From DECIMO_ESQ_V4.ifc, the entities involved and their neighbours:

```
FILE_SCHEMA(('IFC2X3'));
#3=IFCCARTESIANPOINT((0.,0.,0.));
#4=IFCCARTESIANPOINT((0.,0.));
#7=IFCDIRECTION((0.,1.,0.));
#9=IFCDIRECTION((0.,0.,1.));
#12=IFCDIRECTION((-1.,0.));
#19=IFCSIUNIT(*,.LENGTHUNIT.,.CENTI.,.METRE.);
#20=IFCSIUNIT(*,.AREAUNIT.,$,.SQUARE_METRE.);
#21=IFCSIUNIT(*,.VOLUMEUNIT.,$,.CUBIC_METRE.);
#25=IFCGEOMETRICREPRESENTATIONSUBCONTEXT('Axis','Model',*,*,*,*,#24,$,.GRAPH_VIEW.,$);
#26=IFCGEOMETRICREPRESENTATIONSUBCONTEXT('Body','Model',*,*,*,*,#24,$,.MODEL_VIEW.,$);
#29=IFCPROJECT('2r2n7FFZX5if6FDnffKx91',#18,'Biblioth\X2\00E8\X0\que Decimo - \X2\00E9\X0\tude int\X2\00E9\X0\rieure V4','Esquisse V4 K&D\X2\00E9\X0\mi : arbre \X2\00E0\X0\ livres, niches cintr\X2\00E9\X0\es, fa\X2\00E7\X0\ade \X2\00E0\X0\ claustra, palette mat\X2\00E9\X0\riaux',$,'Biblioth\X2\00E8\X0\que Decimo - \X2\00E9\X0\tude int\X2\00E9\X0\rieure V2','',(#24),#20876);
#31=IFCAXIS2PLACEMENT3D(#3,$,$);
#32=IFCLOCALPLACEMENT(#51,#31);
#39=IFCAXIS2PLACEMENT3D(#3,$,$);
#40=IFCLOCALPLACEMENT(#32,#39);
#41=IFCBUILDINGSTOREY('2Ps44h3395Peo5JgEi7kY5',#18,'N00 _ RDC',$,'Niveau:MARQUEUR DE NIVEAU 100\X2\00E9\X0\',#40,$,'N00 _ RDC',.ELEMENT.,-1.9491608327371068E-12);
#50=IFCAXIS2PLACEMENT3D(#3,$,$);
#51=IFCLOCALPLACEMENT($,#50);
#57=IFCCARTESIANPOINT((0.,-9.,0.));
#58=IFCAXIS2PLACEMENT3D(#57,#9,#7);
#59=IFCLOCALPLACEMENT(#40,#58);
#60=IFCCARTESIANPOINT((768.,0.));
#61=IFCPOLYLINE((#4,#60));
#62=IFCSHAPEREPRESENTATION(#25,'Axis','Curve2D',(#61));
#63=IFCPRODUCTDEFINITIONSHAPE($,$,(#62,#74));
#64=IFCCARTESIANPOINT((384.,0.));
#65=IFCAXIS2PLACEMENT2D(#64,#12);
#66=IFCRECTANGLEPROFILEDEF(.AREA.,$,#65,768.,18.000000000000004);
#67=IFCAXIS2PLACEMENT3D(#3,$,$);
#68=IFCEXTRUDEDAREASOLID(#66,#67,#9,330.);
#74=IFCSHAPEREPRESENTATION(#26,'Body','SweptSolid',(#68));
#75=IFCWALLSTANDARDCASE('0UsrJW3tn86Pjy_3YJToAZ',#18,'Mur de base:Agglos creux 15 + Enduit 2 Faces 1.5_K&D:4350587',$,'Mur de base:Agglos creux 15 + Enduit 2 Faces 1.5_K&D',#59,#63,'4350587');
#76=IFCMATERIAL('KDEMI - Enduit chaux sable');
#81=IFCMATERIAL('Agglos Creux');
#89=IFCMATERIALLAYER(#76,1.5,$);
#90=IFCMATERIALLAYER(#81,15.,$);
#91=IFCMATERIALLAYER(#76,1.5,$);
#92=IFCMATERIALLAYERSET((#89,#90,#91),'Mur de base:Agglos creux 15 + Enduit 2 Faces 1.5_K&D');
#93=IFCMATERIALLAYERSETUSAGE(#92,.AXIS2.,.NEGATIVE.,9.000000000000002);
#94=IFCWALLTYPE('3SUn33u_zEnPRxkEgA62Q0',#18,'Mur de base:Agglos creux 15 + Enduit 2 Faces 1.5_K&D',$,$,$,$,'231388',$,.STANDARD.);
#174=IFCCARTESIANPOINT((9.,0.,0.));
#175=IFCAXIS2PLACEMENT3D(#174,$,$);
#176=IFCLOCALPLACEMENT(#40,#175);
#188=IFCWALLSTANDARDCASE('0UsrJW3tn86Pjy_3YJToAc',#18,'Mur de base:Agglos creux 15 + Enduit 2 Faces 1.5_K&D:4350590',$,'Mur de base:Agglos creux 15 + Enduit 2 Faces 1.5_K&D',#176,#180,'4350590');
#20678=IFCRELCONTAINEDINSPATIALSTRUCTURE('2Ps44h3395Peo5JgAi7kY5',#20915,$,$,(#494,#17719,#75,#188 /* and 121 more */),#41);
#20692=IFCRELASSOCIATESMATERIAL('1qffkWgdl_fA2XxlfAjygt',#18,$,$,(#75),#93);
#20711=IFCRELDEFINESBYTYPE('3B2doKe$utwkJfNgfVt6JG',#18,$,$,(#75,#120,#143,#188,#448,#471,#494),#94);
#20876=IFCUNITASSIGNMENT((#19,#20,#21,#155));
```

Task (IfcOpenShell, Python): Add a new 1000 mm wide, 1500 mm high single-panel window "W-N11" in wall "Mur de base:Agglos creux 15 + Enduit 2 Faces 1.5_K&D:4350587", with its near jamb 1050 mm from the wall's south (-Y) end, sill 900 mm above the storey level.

```python
import numpy as np
import ifcopenshell
import ifcopenshell.api.feature
import ifcopenshell.api.geometry
import ifcopenshell.api.root
import ifcopenshell.api.spatial
import ifcopenshell.api.type
import ifcopenshell.geom
import ifcopenshell.util.element
import ifcopenshell.util.placement
import ifcopenshell.util.representation
import ifcopenshell.util.shape
import ifcopenshell.util.unit

model = ifcopenshell.open("DECIMO_ESQ_V4.ifc")
unit_scale = ifcopenshell.util.unit.calculate_unit_scale(model)
settings = ifcopenshell.geom.settings()


def volume(element):
    """Net volume in cubic metres, openings subtracted."""
    shape = ifcopenshell.geom.create_shape(settings, element)
    return ifcopenshell.util.shape.get_volume(shape.geometry)


wall = model.by_guid("0UsrJW3tn86Pjy_3YJToAZ")
storey = ifcopenshell.util.element.get_container(wall, ifc_class="IfcBuildingStorey")
context = ifcopenshell.util.representation.get_context(model, "Model", "Body", "MODEL_VIEW")
before = volume(wall)

width, height, from_end, sill = 1, 1.5, 1.05, 0.9  # metres

# The wall runs along its own X axis, and the end named is its -X end.
wall_shape = ifcopenshell.geom.create_shape(settings, wall)
x, y, z = ifcopenshell.util.shape.get_vertices(wall_shape.geometry).T
start = x.min() + from_end
face, thickness = float(y.min()), float(y.max() - y.min())
wall_matrix = ifcopenshell.util.placement.get_local_placement(wall.ObjectPlacement)
level = ifcopenshell.util.placement.get_local_placement(storey.ObjectPlacement)[2, 3]


def in_wall(x, y):
    """Placement at x, y metres in the wall's axes, at sill height."""
    matrix = wall_matrix.copy()
    matrix[:, 3] = wall_matrix @ np.array([x / unit_scale, y / unit_scale, 0.0, 1.0])
    matrix[2, 3] = level + sill / unit_scale
    return matrix


# Opening: a box that overshoots both wall faces by 50 mm.
opening = ifcopenshell.api.root.create_entity(model, ifc_class="IfcOpeningElement")
box = ifcopenshell.api.geometry.add_wall_representation(
    model, context=context, length=width, height=height, thickness=thickness + 0.1
)
ifcopenshell.api.geometry.assign_representation(model, product=opening, representation=box)
ifcopenshell.api.geometry.edit_object_placement(model, product=opening, matrix=in_wall(start, face - 0.05), is_si=False)
ifcopenshell.api.feature.add_feature(model, feature=opening, element=wall)

window = ifcopenshell.api.root.create_entity(model, ifc_class="IfcWindow", name="W-N11")
window.OverallWidth, window.OverallHeight = width / unit_scale, height / unit_scale
body = ifcopenshell.api.geometry.add_window_representation(
    model,
    context=context,
    overall_width=window.OverallWidth,
    overall_height=window.OverallHeight,
    partition_type="SINGLE_PANEL",
)
ifcopenshell.api.geometry.assign_representation(model, product=window, representation=body)
ifcopenshell.api.spatial.assign_container(model, products=[window], relating_structure=storey)
fills = ifcopenshell.api.feature.add_filling(model, opening=opening, element=window)
fills.OwnerHistory = window.OwnerHistory  # required in IFC2X3

# IFC2X3 keeps the operation on the window style.
style = ifcopenshell.api.root.create_entity(model, ifc_class="IfcWindowStyle", name="W-N11")
style.OperationType, style.ConstructionType = "SINGLE_PANEL", "NOTDEFINED"
style.ParameterTakesPrecedence = style.Sizeable = False
ifcopenshell.api.type.assign_type(model, related_objects=[window], relating_type=style)

# Centre the window in the wall's thickness.
ifcopenshell.api.geometry.edit_object_placement(model, product=window, matrix=in_wall(start, face), is_si=False)
window_shape = ifcopenshell.geom.create_shape(settings, window)
depth = ifcopenshell.util.shape.get_vertices(window_shape.geometry)[:, 1]
offset = face + thickness / 2 - (depth.min() + depth.max()) / 2
ifcopenshell.api.geometry.edit_object_placement(model, product=window, matrix=in_wall(start, offset), is_si=False)

after = volume(wall)

print(f"wall volume {before:.3f} -> {after:.3f} m3")

model.write("DECIMO_ESQ_V4_edited.ifc")
```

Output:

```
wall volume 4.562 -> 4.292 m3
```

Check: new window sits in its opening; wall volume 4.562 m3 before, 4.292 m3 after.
